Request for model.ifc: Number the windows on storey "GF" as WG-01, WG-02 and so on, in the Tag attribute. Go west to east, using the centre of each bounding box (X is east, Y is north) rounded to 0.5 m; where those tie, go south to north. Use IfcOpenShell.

First a look at what the model holds.

```python
import ifcopenshell
import ifcopenshell.util.element
import ifcopenshell.util.placement

model = ifcopenshell.open("model.ifc")
print(model.schema)
storey = next(s for s in model.by_type("IfcBuildingStorey") if s.Name == "GF")
windows = [e for e in ifcopenshell.util.element.get_decomposition(storey) if e.is_a("IfcWindow")]
for e in sorted(windows, key=lambda e: e.id()):
    origin = ifcopenshell.util.placement.get_local_placement(e.ObjectPlacement)[:3, 3]
    print(e.id(), e.Tag, e.Name, origin.round(2) + 0.0, sep=" | ")
```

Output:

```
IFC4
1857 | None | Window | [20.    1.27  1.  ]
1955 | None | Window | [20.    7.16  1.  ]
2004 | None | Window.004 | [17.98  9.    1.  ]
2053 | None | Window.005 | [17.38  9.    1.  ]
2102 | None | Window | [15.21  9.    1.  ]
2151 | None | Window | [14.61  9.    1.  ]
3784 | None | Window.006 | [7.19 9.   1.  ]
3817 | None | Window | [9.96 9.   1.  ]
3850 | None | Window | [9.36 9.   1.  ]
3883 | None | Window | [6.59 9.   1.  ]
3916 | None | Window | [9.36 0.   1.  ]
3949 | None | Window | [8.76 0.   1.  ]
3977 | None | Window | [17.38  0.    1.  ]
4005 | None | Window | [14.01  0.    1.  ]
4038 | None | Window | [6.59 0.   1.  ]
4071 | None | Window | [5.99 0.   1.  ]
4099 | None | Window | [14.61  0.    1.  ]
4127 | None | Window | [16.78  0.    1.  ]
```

```python
import ifcopenshell
import ifcopenshell.geom
import ifcopenshell.util.element
import ifcopenshell.util.shape

model = ifcopenshell.open("model.ifc")
settings = ifcopenshell.geom.settings()
settings.set("use-world-coords", True)


def centre(element):
    shape = ifcopenshell.geom.create_shape(settings, element)
    return ifcopenshell.util.shape.get_bbox_centroid(shape.geometry)


storey = next(s for s in model.by_type("IfcBuildingStorey") if s.Name == "GF")
windows = [e for e in ifcopenshell.util.element.get_decomposition(storey) if e.is_a("IfcWindow")]

# Insertion points can sit at a corner or the storey origin, so sort by the geometry (in metres).
centres = {e: centre(e) for e in windows}
windows.sort(key=lambda e: (round(centres[e][0] / 0.5), centres[e][1]))

for i, e in enumerate(windows, start=1):
    number = f"WG-{i:02d}"
    e.Tag = number
    print(e.id(), number)

model.write("model-out.ifc")
```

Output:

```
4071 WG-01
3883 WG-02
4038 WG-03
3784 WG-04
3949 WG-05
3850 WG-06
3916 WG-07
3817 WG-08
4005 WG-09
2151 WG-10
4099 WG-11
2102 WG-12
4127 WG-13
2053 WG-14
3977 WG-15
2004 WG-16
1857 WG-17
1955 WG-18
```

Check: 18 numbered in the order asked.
